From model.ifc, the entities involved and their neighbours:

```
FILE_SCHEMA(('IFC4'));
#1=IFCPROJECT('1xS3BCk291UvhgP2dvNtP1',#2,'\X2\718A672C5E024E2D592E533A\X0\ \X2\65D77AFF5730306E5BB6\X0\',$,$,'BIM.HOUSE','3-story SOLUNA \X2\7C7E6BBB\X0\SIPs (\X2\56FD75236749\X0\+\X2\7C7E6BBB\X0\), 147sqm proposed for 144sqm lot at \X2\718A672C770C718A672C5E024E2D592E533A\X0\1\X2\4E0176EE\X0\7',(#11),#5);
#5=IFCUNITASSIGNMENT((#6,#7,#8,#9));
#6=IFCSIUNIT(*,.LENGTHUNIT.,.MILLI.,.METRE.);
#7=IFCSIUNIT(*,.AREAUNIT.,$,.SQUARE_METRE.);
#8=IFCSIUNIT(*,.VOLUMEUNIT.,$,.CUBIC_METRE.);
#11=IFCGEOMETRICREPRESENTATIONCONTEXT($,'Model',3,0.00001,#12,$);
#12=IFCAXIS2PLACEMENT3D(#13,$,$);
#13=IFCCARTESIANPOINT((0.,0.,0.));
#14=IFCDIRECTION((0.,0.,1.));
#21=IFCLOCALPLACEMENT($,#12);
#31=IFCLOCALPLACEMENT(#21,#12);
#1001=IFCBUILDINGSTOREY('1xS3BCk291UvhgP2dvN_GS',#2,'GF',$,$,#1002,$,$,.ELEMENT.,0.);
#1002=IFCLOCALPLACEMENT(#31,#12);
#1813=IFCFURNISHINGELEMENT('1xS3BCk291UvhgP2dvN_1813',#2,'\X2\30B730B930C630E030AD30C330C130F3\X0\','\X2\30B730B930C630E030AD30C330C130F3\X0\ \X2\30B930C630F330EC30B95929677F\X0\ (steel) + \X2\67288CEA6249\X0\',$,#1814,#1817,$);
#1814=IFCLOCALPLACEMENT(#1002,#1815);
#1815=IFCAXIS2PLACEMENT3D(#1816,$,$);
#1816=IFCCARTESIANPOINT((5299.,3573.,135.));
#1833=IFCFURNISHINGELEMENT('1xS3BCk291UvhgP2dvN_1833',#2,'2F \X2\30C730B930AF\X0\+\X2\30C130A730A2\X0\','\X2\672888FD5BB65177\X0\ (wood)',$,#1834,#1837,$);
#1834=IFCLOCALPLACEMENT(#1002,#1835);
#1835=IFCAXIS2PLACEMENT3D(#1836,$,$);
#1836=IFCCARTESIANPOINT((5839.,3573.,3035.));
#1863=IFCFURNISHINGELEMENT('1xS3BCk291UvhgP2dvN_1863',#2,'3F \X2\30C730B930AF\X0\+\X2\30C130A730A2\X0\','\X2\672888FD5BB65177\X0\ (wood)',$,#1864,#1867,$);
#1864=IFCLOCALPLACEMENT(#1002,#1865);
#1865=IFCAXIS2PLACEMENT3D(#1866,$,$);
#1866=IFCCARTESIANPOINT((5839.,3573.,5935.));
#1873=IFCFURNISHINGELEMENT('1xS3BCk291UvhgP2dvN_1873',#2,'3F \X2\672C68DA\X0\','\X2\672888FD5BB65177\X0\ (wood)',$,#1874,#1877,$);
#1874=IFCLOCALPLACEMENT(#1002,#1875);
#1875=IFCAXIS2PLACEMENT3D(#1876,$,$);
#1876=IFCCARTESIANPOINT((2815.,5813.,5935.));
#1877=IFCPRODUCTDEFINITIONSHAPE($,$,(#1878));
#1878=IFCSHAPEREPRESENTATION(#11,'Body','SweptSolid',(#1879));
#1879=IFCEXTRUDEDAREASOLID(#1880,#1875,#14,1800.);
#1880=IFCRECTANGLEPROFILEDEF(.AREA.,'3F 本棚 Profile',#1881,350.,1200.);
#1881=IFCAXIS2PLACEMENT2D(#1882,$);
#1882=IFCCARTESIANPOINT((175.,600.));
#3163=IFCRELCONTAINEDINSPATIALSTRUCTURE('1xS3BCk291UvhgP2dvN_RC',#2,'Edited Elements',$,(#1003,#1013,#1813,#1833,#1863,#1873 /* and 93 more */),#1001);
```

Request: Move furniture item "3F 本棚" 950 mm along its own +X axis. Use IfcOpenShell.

```python
import ifcopenshell
import ifcopenshell.api.geometry
import ifcopenshell.util.placement

model = ifcopenshell.open("model.ifc")

item = model.by_guid("1xS3BCk291UvhgP2dvN_1873")
matrix = ifcopenshell.util.placement.get_local_placement(item.ObjectPlacement)
matrix[:3, 3] += matrix[:3, 0] * 950.0
ifcopenshell.api.geometry.edit_object_placement(model, product=item, matrix=matrix, is_si=False)

print(ifcopenshell.util.placement.get_local_placement(item.ObjectPlacement).round(3) + 0.0)

model.write("model_rev.ifc")
```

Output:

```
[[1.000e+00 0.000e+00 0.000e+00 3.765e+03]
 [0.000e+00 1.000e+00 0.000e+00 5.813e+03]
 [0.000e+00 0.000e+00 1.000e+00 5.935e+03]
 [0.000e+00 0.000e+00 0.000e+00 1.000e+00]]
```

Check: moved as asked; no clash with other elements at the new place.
